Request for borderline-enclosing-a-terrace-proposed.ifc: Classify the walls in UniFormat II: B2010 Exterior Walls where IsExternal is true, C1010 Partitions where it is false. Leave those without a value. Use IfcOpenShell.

First a look at what the model holds.

```python
import ifcopenshell
import ifcopenshell.util.element

model = ifcopenshell.open("borderline-enclosing-a-terrace-proposed.ifc")
print(model.schema)
print("classifications:", [c.Name for c in model.by_type("IfcClassification")])
values = [ifcopenshell.util.element.get_pset(e, "Pset_WallCommon", "IsExternal") for e in model.by_type("IfcWall")]
for value in (True, False, None):
    print("IsExternal", value, values.count(value))
```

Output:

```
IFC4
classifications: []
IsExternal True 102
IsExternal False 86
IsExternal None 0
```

```python
import ifcopenshell
import ifcopenshell.api.classification
import ifcopenshell.util.element

model = ifcopenshell.open("borderline-enclosing-a-terrace-proposed.ifc")

system = ifcopenshell.api.classification.add_classification(model, classification="UniFormat II")

walls = model.by_type("IfcWall")
external = {e: ifcopenshell.util.element.get_pset(e, "Pset_WallCommon", "IsExternal") for e in walls}
for flag, code, name in ((True, "B2010", "Exterior Walls"), (False, "C1010", "Partitions")):
    products = [e for e in walls if external[e] is flag]
    ifcopenshell.api.classification.add_reference(
        model, products=products, classification=system, identification=code, name=name
    )
    print(code, len(products))

model.write("borderline-enclosing-a-terrace-proposed_edited.ifc")
```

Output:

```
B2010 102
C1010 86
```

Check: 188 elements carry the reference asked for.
